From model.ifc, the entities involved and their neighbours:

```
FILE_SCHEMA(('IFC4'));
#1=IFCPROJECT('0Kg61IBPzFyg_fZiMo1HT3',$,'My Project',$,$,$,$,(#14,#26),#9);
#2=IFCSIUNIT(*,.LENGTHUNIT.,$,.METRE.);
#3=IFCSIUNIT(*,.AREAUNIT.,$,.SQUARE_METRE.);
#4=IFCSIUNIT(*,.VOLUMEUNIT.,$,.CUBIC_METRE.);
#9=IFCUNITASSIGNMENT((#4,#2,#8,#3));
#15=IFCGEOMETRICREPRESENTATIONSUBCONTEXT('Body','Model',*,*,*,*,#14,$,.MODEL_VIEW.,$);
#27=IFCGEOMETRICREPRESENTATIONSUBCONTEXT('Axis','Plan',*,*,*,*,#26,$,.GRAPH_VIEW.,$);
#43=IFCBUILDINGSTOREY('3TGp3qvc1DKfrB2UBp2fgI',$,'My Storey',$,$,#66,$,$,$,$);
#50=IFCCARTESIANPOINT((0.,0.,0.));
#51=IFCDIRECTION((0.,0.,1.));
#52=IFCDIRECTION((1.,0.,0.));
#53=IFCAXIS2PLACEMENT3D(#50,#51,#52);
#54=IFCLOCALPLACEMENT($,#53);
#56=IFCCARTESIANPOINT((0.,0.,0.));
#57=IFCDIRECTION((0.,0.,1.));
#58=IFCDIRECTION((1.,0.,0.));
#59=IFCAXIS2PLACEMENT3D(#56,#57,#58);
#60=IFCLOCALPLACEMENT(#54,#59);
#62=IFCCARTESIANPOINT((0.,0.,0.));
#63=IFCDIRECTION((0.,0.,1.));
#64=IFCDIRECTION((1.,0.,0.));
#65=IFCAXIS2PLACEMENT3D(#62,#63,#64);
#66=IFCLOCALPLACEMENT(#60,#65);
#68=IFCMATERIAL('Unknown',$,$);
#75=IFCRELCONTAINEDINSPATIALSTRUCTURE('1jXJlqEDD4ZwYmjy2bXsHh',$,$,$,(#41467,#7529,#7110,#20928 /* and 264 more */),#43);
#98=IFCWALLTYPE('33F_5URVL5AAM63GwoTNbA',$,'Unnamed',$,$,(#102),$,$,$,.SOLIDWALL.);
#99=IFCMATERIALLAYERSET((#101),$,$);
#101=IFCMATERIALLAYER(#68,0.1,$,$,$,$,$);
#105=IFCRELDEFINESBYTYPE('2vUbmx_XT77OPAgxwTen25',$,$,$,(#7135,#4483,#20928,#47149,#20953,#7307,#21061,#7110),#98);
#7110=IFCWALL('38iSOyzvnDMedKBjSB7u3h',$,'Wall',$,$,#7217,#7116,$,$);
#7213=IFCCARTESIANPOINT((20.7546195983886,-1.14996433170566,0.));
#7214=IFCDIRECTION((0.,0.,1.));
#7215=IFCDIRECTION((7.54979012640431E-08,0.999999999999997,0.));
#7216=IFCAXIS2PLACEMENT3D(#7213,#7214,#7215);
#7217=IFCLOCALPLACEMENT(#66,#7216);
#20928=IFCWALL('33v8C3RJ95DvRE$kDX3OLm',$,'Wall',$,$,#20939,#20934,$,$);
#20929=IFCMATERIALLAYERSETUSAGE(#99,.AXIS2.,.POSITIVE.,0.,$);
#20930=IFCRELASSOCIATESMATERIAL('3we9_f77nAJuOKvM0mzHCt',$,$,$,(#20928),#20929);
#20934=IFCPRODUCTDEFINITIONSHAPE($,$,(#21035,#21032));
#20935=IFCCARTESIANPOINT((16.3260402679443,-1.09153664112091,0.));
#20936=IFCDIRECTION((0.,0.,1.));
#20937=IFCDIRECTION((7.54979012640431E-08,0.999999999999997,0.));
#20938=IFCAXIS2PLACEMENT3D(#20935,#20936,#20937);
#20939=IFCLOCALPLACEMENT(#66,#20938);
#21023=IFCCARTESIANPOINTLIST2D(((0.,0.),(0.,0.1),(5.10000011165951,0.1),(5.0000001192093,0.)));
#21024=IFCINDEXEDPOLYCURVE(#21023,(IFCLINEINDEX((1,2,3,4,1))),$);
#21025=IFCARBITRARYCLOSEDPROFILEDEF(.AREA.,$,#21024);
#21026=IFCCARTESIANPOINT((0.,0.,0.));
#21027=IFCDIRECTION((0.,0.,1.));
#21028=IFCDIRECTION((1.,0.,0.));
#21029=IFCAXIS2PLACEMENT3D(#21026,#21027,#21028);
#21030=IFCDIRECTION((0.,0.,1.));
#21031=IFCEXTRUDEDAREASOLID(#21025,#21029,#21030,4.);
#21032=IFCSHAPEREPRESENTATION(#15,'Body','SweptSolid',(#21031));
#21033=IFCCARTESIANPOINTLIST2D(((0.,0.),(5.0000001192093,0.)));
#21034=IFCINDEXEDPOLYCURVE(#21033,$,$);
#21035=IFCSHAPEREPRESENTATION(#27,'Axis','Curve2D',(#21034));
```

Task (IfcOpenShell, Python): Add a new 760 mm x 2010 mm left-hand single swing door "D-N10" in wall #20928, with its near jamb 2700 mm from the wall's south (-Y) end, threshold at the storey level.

```python
import numpy as np
import ifcopenshell
import ifcopenshell.api.feature
import ifcopenshell.api.geometry
import ifcopenshell.api.root
import ifcopenshell.api.spatial
import ifcopenshell.geom
import ifcopenshell.util.element
import ifcopenshell.util.placement
import ifcopenshell.util.representation
import ifcopenshell.util.shape
import ifcopenshell.util.unit

model = ifcopenshell.open("model.ifc")
unit_scale = ifcopenshell.util.unit.calculate_unit_scale(model)
settings = ifcopenshell.geom.settings()


def volume(element):
    """Net volume in cubic metres, openings subtracted."""
    shape = ifcopenshell.geom.create_shape(settings, element)
    return ifcopenshell.util.shape.get_volume(shape.geometry)


wall = model.by_guid("33v8C3RJ95DvRE$kDX3OLm")
storey = ifcopenshell.util.element.get_container(wall, ifc_class="IfcBuildingStorey")
context = ifcopenshell.util.representation.get_context(model, "Model", "Body", "MODEL_VIEW")
before = volume(wall)

width, height, from_end, sill = 0.76, 2.01, 2.7, 0.0  # metres

# The wall runs along its own X axis, and the end named is its -X end.
wall_shape = ifcopenshell.geom.create_shape(settings, wall)
x, y, z = ifcopenshell.util.shape.get_vertices(wall_shape.geometry).T
start = x.min() + from_end
face, thickness = float(y.min()), float(y.max() - y.min())
wall_matrix = ifcopenshell.util.placement.get_local_placement(wall.ObjectPlacement)
level = ifcopenshell.util.placement.get_local_placement(storey.ObjectPlacement)[2, 3]


def in_wall(x, y):
    """Placement at x, y metres in the wall's axes, at sill height."""
    matrix = wall_matrix.copy()
    matrix[:, 3] = wall_matrix @ np.array([x / unit_scale, y / unit_scale, 0.0, 1.0])
    matrix[2, 3] = level + sill / unit_scale
    return matrix


# Opening: a box that overshoots both wall faces by 50 mm.
opening = ifcopenshell.api.root.create_entity(model, ifc_class="IfcOpeningElement", predefined_type="OPENING")
box = ifcopenshell.api.geometry.add_wall_representation(
    model, context=context, length=width, height=height, thickness=thickness + 0.1
)
ifcopenshell.api.geometry.assign_representation(model, product=opening, representation=box)
ifcopenshell.api.geometry.edit_object_placement(model, product=opening, matrix=in_wall(start, face - 0.05), is_si=False)
ifcopenshell.api.feature.add_feature(model, feature=opening, element=wall)

door = ifcopenshell.api.root.create_entity(model, ifc_class="IfcDoor", name="D-N10", predefined_type="DOOR")
door.OverallWidth, door.OverallHeight = width / unit_scale, height / unit_scale
door.OperationType = "SINGLE_SWING_LEFT"
body = ifcopenshell.api.geometry.add_door_representation(
    model,
    context=context,
    overall_width=door.OverallWidth,
    overall_height=door.OverallHeight,
    operation_type="SINGLE_SWING_LEFT",
    lining_properties={"LiningDepth": thickness / unit_scale, "ThresholdDepth": thickness / unit_scale},
)
ifcopenshell.api.geometry.assign_representation(model, product=door, representation=body)
ifcopenshell.api.spatial.assign_container(model, products=[door], relating_structure=storey)
ifcopenshell.api.feature.add_filling(model, opening=opening, element=door)

# The lining spans the wall, so the door starts at the wall face.
ifcopenshell.api.geometry.edit_object_placement(model, product=door, matrix=in_wall(start, face), is_si=False)

after = volume(wall)

print(f"wall volume {before:.3f} -> {after:.3f} m3")

model.write("model_updated.ifc")
```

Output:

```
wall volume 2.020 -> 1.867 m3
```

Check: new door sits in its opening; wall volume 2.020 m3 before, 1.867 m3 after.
